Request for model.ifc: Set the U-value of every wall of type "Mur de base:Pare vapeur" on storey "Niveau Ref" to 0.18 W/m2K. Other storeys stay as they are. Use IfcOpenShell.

First a look at what the model holds.

```python
import ifcopenshell
import ifcopenshell.util.element

model = ifcopenshell.open("model.ifc")
print(model.schema)
storey = next(s for s in model.by_type("IfcBuildingStorey") if s.Name == "Niveau Ref")
walls = [e for e in ifcopenshell.util.element.get_decomposition(storey) if e.is_a("IfcWall")]
seen = {}
for e in walls:
    element_type = ifcopenshell.util.element.get_type(e)
    key = (element_type.Name if element_type != e and element_type else None, ifcopenshell.util.element.get_pset(e, "Pset_WallCommon", "ThermalTransmittance"))
    seen[key] = seen.get(key, 0) + 1
for (name, value), count in sorted(seen.items(), key=str):
    print(count, "x", name, "|", value)
```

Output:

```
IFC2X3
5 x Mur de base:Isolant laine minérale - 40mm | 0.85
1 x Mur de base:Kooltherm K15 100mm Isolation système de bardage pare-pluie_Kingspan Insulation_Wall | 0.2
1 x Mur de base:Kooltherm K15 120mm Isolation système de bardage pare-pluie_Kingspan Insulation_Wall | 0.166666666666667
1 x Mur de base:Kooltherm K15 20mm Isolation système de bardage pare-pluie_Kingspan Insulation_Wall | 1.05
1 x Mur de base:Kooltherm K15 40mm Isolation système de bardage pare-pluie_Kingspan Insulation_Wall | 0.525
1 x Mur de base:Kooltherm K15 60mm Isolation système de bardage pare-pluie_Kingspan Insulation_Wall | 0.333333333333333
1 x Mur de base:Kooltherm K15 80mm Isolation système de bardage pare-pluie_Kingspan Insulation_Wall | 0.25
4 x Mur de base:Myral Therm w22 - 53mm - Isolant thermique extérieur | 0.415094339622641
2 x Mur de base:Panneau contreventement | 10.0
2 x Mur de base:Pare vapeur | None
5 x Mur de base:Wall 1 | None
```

```python
import ifcopenshell
import ifcopenshell.api.pset
import ifcopenshell.util.element

model = ifcopenshell.open("model.ifc")

storey = next(s for s in model.by_type("IfcBuildingStorey") if s.Name == "Niveau Ref")
walls = [e for e in ifcopenshell.util.element.get_decomposition(storey) if e.is_a("IfcWall")]

count = 0
for e in walls:
    element_type = ifcopenshell.util.element.get_type(e)
    if element_type in (None, e) or element_type.Name != "Mur de base:Pare vapeur":
        continue
    # add_pset returns the element's existing set when there is one.
    pset = ifcopenshell.api.pset.add_pset(model, product=e, name="Pset_WallCommon")
    ifcopenshell.api.pset.edit_pset(model, pset=pset, properties={"ThermalTransmittance": 0.18})
    count += 1

print(count, "walls updated")

model.write("model_edited.ifc")
```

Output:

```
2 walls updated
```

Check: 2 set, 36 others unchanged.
